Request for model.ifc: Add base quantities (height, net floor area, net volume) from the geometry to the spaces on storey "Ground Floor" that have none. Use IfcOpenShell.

First a look at what the model holds.

```python
import ifcopenshell
import ifcopenshell.util.element
import ifcopenshell.util.unit

model = ifcopenshell.open("model.ifc")
print(model.schema)
for unit_type in ("LENGTHUNIT", "AREAUNIT", "VOLUMEUNIT"):
    print(unit_type, ifcopenshell.util.unit.calculate_unit_scale(model, unit_type))
storey = next(s for s in model.by_type("IfcBuildingStorey") if s.Name == "Ground Floor")
spaces = [e for e in ifcopenshell.util.element.get_decomposition(storey) if e.is_a("IfcSpace")]
for e in sorted(spaces, key=lambda e: e.id()):
    print(e.id(), e.is_a(), e.Name, list(ifcopenshell.util.element.get_psets(e, qtos_only=True)), sep=" | ")
```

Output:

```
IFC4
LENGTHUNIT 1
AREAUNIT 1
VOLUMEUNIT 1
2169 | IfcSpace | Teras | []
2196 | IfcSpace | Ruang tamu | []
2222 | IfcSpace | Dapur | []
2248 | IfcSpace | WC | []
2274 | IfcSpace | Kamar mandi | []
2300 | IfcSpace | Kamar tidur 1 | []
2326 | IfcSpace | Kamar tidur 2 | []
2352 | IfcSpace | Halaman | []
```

```python
import ifcopenshell
import ifcopenshell.api.pset
import ifcopenshell.geom
import ifcopenshell.util.element
import ifcopenshell.util.shape
import ifcopenshell.util.unit

model = ifcopenshell.open("model.ifc")
unit_scale = ifcopenshell.util.unit.calculate_unit_scale(model)
area_scale = ifcopenshell.util.unit.calculate_unit_scale(model, "AREAUNIT")
volume_scale = ifcopenshell.util.unit.calculate_unit_scale(model, "VOLUMEUNIT")
settings = ifcopenshell.geom.settings()

storey = next(s for s in model.by_type("IfcBuildingStorey") if s.Name == "Ground Floor")
spaces = [e for e in ifcopenshell.util.element.get_decomposition(storey) if e.is_a("IfcSpace")]

for e in sorted(spaces, key=lambda e: e.id()):
    if ifcopenshell.util.element.get_psets(e, qtos_only=True, should_inherit=False):
        continue
    # Geometry comes back in metres, in the element's own axes.
    shape = ifcopenshell.geom.create_shape(settings, e)
    values = {
        "Height": ifcopenshell.util.shape.get_z(shape.geometry) / unit_scale,
        "NetFloorArea": ifcopenshell.util.shape.get_footprint_area(shape.geometry) / area_scale,
        "NetVolume": ifcopenshell.util.shape.get_volume(shape.geometry) / volume_scale,
    }
    qto = ifcopenshell.api.pset.add_qto(model, product=e, name="Qto_SpaceBaseQuantities")
    ifcopenshell.api.pset.edit_qto(model, qto=qto, properties=values)
    print(e.id(), {k: round(v, 3) for k, v in values.items()})

model.write("model_v2.ifc")
```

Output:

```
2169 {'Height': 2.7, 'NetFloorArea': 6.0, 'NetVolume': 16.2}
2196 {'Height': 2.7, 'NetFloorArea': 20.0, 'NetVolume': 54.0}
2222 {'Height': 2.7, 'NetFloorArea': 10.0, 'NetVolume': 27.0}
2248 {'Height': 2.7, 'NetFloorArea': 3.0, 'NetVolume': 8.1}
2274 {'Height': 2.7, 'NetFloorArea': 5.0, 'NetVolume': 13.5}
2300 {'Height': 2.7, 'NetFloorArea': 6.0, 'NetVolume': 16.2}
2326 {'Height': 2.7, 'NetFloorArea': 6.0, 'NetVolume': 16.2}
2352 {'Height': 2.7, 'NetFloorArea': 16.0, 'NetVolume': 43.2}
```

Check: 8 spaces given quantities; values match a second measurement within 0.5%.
